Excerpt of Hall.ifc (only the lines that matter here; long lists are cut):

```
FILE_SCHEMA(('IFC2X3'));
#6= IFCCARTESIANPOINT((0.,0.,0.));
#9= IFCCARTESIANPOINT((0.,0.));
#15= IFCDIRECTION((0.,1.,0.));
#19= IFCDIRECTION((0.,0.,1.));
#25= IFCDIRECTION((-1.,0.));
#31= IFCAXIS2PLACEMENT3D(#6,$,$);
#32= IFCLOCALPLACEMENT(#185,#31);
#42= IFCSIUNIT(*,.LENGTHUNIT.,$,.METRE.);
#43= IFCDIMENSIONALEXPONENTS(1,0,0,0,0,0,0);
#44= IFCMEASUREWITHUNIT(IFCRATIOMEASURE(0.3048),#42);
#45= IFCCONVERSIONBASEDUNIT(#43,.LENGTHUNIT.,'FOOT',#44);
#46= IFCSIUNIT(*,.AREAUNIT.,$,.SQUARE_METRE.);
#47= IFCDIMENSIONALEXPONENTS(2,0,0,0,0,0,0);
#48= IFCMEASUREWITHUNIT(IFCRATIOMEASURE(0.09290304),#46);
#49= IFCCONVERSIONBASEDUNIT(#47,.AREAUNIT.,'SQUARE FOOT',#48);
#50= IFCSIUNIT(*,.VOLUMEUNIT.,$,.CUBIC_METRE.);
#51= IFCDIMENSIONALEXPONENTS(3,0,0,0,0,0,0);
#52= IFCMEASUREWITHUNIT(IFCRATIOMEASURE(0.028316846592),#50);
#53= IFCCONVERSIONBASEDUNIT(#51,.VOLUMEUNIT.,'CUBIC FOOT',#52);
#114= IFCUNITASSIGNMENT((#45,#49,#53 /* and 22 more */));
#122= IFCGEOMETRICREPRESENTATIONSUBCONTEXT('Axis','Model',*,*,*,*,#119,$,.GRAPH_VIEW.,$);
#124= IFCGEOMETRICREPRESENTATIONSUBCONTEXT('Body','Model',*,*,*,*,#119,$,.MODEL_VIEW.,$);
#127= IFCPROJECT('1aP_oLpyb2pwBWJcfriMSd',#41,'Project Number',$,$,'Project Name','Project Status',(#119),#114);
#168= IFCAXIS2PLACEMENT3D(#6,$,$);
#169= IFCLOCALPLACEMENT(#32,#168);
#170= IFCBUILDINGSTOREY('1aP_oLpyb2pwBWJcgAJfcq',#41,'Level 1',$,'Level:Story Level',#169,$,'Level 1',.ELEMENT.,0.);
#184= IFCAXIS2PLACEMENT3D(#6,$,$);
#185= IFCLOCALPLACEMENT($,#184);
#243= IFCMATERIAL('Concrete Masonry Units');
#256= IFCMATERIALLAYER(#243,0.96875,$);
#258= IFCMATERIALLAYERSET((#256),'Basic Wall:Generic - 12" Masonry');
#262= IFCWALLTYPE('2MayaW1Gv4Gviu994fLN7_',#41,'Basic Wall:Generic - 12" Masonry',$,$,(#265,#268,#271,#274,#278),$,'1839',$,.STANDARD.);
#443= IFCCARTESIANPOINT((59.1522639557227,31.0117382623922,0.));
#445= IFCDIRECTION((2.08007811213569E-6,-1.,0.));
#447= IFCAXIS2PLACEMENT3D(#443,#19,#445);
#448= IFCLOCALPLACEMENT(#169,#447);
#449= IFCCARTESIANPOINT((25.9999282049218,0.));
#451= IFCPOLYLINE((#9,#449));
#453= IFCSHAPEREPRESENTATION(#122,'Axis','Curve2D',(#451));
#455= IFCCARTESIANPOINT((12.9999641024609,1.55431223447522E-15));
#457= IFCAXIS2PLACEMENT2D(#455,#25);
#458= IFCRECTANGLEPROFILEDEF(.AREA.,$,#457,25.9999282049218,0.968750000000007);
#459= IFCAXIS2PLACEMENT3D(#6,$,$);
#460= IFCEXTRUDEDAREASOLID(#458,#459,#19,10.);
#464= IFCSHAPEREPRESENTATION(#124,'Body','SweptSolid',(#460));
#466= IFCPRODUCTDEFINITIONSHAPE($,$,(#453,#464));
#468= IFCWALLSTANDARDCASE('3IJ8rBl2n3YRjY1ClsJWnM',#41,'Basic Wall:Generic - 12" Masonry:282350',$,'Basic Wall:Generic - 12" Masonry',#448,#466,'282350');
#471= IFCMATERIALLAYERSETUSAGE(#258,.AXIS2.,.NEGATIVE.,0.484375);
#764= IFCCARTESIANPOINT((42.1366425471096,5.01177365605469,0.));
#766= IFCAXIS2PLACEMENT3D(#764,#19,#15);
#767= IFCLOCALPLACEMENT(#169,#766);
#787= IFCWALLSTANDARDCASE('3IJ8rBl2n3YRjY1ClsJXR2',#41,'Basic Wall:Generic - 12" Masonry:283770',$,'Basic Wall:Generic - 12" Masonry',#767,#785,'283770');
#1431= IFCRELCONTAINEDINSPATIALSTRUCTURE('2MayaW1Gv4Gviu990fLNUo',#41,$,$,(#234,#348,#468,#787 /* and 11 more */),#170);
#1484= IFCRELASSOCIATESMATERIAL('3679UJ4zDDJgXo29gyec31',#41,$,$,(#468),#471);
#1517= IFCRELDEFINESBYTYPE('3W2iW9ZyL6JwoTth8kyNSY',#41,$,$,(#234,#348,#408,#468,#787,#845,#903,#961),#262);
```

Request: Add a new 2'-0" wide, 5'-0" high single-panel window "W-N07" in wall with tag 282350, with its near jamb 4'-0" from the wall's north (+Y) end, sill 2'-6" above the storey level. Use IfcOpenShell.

```python
import numpy as np
import ifcopenshell
import ifcopenshell.api.feature
import ifcopenshell.api.geometry
import ifcopenshell.api.root
import ifcopenshell.api.spatial
import ifcopenshell.api.type
import ifcopenshell.geom
import ifcopenshell.util.element
import ifcopenshell.util.placement
import ifcopenshell.util.representation
import ifcopenshell.util.shape
import ifcopenshell.util.unit

model = ifcopenshell.open("Hall.ifc")
unit_scale = ifcopenshell.util.unit.calculate_unit_scale(model)
settings = ifcopenshell.geom.settings()


def volume(element):
    """Net volume in cubic metres, openings subtracted."""
    shape = ifcopenshell.geom.create_shape(settings, element)
    return ifcopenshell.util.shape.get_volume(shape.geometry)


wall = model.by_guid("3IJ8rBl2n3YRjY1ClsJWnM")
storey = ifcopenshell.util.element.get_container(wall, ifc_class="IfcBuildingStorey")
context = ifcopenshell.util.representation.get_context(model, "Model", "Body", "MODEL_VIEW")
before = volume(wall)

width, height, from_end, sill = 0.6096, 1.524, 1.2192, 0.762  # metres

# The wall runs along its own X axis, and the end named is its -X end.
wall_shape = ifcopenshell.geom.create_shape(settings, wall)
x, y, z = ifcopenshell.util.shape.get_vertices(wall_shape.geometry).T
start = x.min() + from_end
face, thickness = float(y.min()), float(y.max() - y.min())
wall_matrix = ifcopenshell.util.placement.get_local_placement(wall.ObjectPlacement)
level = ifcopenshell.util.placement.get_local_placement(storey.ObjectPlacement)[2, 3]


def in_wall(x, y):
    """Placement at x, y metres in the wall's axes, at sill height."""
    matrix = wall_matrix.copy()
    matrix[:, 3] = wall_matrix @ np.array([x / unit_scale, y / unit_scale, 0.0, 1.0])
    matrix[2, 3] = level + sill / unit_scale
    return matrix


# Opening: a box that overshoots both wall faces by 50 mm.
opening = ifcopenshell.api.root.create_entity(model, ifc_class="IfcOpeningElement")
box = ifcopenshell.api.geometry.add_wall_representation(
    model, context=context, length=width, height=height, thickness=thickness + 0.1
)
ifcopenshell.api.geometry.assign_representation(model, product=opening, representation=box)
ifcopenshell.api.geometry.edit_object_placement(model, product=opening, matrix=in_wall(start, face - 0.05), is_si=False)
ifcopenshell.api.feature.add_feature(model, feature=opening, element=wall)

window = ifcopenshell.api.root.create_entity(model, ifc_class="IfcWindow", name="W-N07")
window.OverallWidth, window.OverallHeight = width / unit_scale, height / unit_scale
body = ifcopenshell.api.geometry.add_window_representation(
    model,
    context=context,
    overall_width=window.OverallWidth,
    overall_height=window.OverallHeight,
    partition_type="SINGLE_PANEL",
)
ifcopenshell.api.geometry.assign_representation(model, product=window, representation=body)
ifcopenshell.api.spatial.assign_container(model, products=[window], relating_structure=storey)
fills = ifcopenshell.api.feature.add_filling(model, opening=opening, element=window)
fills.OwnerHistory = window.OwnerHistory  # required in IFC2X3

# IFC2X3 keeps the operation on the window style.
style = ifcopenshell.api.root.create_entity(model, ifc_class="IfcWindowStyle", name="W-N07")
style.OperationType, style.ConstructionType = "SINGLE_PANEL", "NOTDEFINED"
style.ParameterTakesPrecedence = style.Sizeable = False
ifcopenshell.api.type.assign_type(model, related_objects=[window], relating_type=style)

# Centre the window in the wall's thickness.
ifcopenshell.api.geometry.edit_object_placement(model, product=window, matrix=in_wall(start, face), is_si=False)
window_shape = ifcopenshell.geom.create_shape(settings, window)
depth = ifcopenshell.util.shape.get_vertices(window_shape.geometry)[:, 1]
offset = face + thickness / 2 - (depth.min() + depth.max()) / 2
ifcopenshell.api.geometry.edit_object_placement(model, product=window, matrix=in_wall(start, offset), is_si=False)

after = volume(wall)

print(f"wall volume {before:.3f} -> {after:.3f} m3")

model.write("Hall_updated.ifc")
```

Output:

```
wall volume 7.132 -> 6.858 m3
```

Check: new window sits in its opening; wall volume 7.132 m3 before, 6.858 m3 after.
